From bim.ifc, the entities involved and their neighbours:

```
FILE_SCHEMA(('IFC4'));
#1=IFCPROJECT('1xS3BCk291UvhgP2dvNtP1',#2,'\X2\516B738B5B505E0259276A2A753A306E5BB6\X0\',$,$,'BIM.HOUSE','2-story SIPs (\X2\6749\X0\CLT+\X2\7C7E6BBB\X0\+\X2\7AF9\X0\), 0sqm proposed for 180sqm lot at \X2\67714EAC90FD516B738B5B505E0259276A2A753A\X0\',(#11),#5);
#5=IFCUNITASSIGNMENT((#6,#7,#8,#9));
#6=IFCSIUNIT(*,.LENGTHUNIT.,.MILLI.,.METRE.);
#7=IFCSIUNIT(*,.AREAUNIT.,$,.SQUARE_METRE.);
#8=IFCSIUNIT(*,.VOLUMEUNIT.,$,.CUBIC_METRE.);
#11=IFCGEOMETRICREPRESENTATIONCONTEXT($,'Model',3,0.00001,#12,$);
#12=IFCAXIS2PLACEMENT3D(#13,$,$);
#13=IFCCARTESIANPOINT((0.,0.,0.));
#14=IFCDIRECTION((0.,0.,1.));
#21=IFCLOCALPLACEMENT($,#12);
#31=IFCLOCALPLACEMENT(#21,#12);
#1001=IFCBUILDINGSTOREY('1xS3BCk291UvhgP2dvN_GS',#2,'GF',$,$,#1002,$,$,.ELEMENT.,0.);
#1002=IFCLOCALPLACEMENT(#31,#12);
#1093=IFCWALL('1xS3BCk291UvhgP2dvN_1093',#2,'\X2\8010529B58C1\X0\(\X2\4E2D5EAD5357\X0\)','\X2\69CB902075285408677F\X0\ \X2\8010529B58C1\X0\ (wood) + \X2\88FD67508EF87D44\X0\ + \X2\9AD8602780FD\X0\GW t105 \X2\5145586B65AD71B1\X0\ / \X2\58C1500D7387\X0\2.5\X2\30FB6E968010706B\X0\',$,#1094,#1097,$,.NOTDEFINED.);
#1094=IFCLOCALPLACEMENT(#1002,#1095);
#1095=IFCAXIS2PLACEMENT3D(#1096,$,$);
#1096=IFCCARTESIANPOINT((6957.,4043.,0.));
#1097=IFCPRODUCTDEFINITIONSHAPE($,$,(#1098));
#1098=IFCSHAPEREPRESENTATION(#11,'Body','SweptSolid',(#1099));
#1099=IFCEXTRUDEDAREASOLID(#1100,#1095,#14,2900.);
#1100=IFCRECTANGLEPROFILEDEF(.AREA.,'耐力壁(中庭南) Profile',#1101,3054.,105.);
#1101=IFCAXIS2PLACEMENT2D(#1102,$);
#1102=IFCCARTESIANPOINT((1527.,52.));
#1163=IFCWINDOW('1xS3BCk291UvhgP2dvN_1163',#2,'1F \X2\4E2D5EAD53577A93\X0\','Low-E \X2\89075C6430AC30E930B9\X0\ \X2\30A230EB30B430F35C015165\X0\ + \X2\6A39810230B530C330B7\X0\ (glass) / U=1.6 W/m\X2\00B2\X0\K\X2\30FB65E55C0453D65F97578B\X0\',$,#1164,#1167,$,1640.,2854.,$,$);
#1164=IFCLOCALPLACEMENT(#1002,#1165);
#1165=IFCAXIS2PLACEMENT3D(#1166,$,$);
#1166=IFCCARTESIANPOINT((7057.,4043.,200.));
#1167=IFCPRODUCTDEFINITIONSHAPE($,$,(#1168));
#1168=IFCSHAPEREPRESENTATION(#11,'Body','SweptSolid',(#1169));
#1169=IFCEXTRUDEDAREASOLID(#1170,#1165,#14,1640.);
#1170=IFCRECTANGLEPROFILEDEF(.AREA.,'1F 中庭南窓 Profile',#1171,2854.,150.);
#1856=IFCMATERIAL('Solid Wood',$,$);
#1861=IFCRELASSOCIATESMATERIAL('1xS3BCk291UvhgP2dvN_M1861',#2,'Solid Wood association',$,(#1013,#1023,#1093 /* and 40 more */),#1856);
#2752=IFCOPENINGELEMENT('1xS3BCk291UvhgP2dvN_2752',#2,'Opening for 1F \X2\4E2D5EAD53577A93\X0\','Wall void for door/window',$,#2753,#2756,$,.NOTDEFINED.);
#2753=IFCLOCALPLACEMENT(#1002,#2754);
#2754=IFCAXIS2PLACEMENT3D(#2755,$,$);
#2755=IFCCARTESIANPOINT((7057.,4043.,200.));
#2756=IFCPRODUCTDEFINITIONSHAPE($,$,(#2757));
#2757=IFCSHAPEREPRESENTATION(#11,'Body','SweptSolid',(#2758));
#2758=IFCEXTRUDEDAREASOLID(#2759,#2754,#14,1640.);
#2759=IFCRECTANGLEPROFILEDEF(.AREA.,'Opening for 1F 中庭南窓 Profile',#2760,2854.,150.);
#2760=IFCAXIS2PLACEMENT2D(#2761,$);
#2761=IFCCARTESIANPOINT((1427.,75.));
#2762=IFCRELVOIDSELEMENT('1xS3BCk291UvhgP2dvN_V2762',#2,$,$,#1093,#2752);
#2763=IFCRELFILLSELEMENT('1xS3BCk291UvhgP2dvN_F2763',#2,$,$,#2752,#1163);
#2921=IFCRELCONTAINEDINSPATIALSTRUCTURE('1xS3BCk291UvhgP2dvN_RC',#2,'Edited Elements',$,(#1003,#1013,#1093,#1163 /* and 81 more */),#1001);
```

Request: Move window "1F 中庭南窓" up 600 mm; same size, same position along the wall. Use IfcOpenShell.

```python
import numpy as np
import ifcopenshell
import ifcopenshell.api.geometry
import ifcopenshell.util.placement
import ifcopenshell.util.unit

model = ifcopenshell.open("bim.ifc")
unit_scale = ifcopenshell.util.unit.calculate_unit_scale(model)

window = model.by_guid("1xS3BCk291UvhgP2dvN_1163")
opening = window.FillsVoids[0].RelatingOpeningElement
dz = 600.0

shift = np.array([0.0, 0.0, dz])
# The window is not placed relative to its opening, so move both.
for product in (opening, window):
    matrix = ifcopenshell.util.placement.get_local_placement(product.ObjectPlacement)
    matrix[:3, 3] += shift
    ifcopenshell.api.geometry.edit_object_placement(model, product=product, matrix=matrix, is_si=False)

print(f"moved by {dz * unit_scale:+.3f} m")

model.write("bim-out.ifc")
```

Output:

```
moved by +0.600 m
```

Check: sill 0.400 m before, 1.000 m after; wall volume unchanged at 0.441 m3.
